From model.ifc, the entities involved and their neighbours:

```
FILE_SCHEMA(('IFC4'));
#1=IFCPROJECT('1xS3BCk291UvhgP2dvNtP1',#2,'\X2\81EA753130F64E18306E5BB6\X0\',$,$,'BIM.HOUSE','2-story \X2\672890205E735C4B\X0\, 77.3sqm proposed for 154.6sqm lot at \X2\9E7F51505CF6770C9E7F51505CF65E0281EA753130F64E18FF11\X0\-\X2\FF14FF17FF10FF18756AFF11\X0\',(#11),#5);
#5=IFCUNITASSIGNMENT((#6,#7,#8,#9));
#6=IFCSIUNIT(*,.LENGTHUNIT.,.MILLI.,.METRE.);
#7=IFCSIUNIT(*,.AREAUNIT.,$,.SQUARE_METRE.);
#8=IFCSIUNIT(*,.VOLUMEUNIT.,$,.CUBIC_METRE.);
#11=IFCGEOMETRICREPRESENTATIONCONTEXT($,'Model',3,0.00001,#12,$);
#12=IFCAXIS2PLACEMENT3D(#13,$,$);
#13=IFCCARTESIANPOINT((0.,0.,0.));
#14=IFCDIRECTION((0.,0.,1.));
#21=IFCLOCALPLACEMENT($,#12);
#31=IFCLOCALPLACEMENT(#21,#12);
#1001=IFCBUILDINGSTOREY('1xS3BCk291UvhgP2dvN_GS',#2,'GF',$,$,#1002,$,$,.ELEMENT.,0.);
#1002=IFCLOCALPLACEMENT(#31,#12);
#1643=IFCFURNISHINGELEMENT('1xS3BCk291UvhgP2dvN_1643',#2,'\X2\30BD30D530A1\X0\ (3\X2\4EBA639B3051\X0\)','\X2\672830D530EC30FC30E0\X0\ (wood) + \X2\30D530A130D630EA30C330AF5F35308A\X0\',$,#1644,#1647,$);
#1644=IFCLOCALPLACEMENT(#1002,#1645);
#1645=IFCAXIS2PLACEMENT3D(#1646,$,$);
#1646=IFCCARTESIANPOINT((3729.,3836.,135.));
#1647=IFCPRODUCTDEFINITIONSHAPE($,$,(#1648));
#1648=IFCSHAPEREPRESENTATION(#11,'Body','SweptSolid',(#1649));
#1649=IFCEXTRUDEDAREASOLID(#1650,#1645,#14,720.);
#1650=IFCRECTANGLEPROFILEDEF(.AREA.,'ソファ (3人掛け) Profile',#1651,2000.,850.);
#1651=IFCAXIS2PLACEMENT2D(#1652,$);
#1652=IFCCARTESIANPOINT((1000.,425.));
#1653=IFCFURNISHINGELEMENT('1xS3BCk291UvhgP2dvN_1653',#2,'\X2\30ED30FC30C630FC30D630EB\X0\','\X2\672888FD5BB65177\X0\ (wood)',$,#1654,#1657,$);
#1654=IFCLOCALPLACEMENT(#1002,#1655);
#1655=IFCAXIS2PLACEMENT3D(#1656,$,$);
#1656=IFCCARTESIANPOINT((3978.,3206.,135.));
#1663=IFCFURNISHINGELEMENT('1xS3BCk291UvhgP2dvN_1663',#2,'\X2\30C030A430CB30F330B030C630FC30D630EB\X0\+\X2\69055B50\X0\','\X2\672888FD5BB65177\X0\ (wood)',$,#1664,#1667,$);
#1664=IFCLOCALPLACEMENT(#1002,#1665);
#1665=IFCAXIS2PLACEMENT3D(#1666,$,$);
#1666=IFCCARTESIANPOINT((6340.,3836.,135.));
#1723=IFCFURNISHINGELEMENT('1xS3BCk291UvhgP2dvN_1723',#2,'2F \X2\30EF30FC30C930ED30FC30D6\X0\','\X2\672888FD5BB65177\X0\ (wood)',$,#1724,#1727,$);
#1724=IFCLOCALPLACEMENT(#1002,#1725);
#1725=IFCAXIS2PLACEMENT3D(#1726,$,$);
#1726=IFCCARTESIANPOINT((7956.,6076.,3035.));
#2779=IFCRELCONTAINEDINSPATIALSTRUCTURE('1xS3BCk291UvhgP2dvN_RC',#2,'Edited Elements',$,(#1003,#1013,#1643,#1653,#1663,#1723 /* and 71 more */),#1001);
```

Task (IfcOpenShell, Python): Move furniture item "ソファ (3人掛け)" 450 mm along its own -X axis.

```python
import ifcopenshell
import ifcopenshell.api.geometry
import ifcopenshell.util.placement
import ifcopenshell.util.unit

model = ifcopenshell.open("model.ifc")
unit_scale = ifcopenshell.util.unit.calculate_unit_scale(model)

item = model.by_id(1643)
matrix = ifcopenshell.util.placement.get_local_placement(item.ObjectPlacement)
matrix[:3, 3] -= matrix[:3, 0] * 0.45 / unit_scale
ifcopenshell.api.geometry.edit_object_placement(model, product=item, matrix=matrix, is_si=False)

print(ifcopenshell.util.placement.get_local_placement(item.ObjectPlacement).round(3) + 0.0)

model.write("model-out.ifc")
```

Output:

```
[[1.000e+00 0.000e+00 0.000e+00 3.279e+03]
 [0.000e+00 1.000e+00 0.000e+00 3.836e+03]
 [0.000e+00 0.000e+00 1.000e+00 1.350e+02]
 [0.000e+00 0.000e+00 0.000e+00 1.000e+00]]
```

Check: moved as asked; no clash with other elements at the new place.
